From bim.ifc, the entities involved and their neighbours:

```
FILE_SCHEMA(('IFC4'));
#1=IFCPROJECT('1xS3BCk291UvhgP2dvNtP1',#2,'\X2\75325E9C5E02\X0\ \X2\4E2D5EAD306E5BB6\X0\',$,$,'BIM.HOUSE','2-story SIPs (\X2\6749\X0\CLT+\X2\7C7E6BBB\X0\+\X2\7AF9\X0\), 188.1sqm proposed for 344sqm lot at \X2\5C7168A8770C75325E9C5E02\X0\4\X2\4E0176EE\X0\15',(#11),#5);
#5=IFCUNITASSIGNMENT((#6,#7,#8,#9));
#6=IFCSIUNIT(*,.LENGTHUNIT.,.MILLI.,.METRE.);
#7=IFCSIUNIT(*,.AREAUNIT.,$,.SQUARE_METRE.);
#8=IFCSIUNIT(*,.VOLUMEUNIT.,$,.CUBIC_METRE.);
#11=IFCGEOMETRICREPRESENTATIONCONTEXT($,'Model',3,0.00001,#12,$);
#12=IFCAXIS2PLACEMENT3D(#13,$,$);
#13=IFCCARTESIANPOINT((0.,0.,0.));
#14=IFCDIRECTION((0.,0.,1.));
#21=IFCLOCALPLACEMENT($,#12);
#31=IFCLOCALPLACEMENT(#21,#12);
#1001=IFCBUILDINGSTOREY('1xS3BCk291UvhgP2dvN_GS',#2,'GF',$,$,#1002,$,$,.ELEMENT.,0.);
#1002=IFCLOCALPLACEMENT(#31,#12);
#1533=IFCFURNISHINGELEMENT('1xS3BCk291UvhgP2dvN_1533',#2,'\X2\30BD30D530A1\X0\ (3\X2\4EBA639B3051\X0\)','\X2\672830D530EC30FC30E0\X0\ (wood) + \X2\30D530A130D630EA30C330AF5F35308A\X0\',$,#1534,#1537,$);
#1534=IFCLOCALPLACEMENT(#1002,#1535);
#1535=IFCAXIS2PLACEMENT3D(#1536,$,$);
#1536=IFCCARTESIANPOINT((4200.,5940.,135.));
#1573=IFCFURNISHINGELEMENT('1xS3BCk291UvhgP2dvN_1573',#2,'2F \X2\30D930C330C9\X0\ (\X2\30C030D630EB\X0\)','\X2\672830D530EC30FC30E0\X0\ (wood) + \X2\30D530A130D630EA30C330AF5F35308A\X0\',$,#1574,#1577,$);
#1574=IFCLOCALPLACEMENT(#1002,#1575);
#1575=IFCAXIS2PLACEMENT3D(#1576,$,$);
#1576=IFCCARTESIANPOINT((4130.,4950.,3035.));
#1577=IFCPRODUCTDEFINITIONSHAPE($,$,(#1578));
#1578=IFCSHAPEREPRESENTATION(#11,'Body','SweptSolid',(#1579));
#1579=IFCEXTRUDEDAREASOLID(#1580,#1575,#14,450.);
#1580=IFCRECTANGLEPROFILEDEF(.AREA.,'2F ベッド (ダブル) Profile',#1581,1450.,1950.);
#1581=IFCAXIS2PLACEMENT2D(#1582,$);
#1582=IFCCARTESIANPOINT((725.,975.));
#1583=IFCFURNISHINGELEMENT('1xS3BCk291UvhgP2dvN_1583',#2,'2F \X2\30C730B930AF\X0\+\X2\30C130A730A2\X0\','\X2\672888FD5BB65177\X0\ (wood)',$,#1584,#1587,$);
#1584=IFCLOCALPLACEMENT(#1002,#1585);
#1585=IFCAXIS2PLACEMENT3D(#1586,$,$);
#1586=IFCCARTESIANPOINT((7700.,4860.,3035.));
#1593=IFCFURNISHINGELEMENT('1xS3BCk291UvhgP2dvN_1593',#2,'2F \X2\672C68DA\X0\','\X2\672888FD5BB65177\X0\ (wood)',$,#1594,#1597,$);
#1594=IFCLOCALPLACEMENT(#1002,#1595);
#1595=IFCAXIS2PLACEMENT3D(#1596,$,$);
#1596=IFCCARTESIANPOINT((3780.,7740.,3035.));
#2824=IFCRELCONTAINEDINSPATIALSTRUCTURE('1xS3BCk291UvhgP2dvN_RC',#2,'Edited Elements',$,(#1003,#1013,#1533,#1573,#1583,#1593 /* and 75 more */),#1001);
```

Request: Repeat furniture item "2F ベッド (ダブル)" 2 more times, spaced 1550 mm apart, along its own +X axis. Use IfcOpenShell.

```python
import ifcopenshell
import ifcopenshell.api.geometry
import ifcopenshell.api.root
import ifcopenshell.util.element
import ifcopenshell.util.placement
import ifcopenshell.util.unit

model = ifcopenshell.open("bim.ifc")
unit_scale = ifcopenshell.util.unit.calculate_unit_scale(model)


def reuse_history(source, copy):
    """copy_class also copies each property set's owner history, people and application; keep the originals."""
    for rel in copy.IsDefinedBy:
        if rel.is_a("IfcRelDefinesByProperties") and (history := rel.RelatingPropertyDefinition.OwnerHistory):
            rel.RelatingPropertyDefinition.OwnerHistory = source.OwnerHistory
            ifcopenshell.util.element.remove_deep2(model, history)


source = model.by_guid("1xS3BCk291UvhgP2dvN_1573")
base = ifcopenshell.util.placement.get_local_placement(source.ObjectPlacement)
step = base[:3, 0] * 1.55 / unit_scale

for i in range(1, 3):
    copy = ifcopenshell.api.root.copy_class(model, product=source)
    copy.Representation = ifcopenshell.util.element.copy_deep(
        model, source.Representation, exclude=["IfcGeometricRepresentationContext", "IfcRepresentationMap"]
    )
    reuse_history(source, copy)
    matrix = base.copy()
    matrix[:3, 3] += i * step
    print("added at", matrix[:3, 3].round(3) + 0.0)
    ifcopenshell.api.geometry.edit_object_placement(model, product=copy, matrix=matrix, is_si=False)

model.write("bim_updated.ifc")
```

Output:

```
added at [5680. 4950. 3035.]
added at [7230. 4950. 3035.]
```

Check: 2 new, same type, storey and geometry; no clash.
